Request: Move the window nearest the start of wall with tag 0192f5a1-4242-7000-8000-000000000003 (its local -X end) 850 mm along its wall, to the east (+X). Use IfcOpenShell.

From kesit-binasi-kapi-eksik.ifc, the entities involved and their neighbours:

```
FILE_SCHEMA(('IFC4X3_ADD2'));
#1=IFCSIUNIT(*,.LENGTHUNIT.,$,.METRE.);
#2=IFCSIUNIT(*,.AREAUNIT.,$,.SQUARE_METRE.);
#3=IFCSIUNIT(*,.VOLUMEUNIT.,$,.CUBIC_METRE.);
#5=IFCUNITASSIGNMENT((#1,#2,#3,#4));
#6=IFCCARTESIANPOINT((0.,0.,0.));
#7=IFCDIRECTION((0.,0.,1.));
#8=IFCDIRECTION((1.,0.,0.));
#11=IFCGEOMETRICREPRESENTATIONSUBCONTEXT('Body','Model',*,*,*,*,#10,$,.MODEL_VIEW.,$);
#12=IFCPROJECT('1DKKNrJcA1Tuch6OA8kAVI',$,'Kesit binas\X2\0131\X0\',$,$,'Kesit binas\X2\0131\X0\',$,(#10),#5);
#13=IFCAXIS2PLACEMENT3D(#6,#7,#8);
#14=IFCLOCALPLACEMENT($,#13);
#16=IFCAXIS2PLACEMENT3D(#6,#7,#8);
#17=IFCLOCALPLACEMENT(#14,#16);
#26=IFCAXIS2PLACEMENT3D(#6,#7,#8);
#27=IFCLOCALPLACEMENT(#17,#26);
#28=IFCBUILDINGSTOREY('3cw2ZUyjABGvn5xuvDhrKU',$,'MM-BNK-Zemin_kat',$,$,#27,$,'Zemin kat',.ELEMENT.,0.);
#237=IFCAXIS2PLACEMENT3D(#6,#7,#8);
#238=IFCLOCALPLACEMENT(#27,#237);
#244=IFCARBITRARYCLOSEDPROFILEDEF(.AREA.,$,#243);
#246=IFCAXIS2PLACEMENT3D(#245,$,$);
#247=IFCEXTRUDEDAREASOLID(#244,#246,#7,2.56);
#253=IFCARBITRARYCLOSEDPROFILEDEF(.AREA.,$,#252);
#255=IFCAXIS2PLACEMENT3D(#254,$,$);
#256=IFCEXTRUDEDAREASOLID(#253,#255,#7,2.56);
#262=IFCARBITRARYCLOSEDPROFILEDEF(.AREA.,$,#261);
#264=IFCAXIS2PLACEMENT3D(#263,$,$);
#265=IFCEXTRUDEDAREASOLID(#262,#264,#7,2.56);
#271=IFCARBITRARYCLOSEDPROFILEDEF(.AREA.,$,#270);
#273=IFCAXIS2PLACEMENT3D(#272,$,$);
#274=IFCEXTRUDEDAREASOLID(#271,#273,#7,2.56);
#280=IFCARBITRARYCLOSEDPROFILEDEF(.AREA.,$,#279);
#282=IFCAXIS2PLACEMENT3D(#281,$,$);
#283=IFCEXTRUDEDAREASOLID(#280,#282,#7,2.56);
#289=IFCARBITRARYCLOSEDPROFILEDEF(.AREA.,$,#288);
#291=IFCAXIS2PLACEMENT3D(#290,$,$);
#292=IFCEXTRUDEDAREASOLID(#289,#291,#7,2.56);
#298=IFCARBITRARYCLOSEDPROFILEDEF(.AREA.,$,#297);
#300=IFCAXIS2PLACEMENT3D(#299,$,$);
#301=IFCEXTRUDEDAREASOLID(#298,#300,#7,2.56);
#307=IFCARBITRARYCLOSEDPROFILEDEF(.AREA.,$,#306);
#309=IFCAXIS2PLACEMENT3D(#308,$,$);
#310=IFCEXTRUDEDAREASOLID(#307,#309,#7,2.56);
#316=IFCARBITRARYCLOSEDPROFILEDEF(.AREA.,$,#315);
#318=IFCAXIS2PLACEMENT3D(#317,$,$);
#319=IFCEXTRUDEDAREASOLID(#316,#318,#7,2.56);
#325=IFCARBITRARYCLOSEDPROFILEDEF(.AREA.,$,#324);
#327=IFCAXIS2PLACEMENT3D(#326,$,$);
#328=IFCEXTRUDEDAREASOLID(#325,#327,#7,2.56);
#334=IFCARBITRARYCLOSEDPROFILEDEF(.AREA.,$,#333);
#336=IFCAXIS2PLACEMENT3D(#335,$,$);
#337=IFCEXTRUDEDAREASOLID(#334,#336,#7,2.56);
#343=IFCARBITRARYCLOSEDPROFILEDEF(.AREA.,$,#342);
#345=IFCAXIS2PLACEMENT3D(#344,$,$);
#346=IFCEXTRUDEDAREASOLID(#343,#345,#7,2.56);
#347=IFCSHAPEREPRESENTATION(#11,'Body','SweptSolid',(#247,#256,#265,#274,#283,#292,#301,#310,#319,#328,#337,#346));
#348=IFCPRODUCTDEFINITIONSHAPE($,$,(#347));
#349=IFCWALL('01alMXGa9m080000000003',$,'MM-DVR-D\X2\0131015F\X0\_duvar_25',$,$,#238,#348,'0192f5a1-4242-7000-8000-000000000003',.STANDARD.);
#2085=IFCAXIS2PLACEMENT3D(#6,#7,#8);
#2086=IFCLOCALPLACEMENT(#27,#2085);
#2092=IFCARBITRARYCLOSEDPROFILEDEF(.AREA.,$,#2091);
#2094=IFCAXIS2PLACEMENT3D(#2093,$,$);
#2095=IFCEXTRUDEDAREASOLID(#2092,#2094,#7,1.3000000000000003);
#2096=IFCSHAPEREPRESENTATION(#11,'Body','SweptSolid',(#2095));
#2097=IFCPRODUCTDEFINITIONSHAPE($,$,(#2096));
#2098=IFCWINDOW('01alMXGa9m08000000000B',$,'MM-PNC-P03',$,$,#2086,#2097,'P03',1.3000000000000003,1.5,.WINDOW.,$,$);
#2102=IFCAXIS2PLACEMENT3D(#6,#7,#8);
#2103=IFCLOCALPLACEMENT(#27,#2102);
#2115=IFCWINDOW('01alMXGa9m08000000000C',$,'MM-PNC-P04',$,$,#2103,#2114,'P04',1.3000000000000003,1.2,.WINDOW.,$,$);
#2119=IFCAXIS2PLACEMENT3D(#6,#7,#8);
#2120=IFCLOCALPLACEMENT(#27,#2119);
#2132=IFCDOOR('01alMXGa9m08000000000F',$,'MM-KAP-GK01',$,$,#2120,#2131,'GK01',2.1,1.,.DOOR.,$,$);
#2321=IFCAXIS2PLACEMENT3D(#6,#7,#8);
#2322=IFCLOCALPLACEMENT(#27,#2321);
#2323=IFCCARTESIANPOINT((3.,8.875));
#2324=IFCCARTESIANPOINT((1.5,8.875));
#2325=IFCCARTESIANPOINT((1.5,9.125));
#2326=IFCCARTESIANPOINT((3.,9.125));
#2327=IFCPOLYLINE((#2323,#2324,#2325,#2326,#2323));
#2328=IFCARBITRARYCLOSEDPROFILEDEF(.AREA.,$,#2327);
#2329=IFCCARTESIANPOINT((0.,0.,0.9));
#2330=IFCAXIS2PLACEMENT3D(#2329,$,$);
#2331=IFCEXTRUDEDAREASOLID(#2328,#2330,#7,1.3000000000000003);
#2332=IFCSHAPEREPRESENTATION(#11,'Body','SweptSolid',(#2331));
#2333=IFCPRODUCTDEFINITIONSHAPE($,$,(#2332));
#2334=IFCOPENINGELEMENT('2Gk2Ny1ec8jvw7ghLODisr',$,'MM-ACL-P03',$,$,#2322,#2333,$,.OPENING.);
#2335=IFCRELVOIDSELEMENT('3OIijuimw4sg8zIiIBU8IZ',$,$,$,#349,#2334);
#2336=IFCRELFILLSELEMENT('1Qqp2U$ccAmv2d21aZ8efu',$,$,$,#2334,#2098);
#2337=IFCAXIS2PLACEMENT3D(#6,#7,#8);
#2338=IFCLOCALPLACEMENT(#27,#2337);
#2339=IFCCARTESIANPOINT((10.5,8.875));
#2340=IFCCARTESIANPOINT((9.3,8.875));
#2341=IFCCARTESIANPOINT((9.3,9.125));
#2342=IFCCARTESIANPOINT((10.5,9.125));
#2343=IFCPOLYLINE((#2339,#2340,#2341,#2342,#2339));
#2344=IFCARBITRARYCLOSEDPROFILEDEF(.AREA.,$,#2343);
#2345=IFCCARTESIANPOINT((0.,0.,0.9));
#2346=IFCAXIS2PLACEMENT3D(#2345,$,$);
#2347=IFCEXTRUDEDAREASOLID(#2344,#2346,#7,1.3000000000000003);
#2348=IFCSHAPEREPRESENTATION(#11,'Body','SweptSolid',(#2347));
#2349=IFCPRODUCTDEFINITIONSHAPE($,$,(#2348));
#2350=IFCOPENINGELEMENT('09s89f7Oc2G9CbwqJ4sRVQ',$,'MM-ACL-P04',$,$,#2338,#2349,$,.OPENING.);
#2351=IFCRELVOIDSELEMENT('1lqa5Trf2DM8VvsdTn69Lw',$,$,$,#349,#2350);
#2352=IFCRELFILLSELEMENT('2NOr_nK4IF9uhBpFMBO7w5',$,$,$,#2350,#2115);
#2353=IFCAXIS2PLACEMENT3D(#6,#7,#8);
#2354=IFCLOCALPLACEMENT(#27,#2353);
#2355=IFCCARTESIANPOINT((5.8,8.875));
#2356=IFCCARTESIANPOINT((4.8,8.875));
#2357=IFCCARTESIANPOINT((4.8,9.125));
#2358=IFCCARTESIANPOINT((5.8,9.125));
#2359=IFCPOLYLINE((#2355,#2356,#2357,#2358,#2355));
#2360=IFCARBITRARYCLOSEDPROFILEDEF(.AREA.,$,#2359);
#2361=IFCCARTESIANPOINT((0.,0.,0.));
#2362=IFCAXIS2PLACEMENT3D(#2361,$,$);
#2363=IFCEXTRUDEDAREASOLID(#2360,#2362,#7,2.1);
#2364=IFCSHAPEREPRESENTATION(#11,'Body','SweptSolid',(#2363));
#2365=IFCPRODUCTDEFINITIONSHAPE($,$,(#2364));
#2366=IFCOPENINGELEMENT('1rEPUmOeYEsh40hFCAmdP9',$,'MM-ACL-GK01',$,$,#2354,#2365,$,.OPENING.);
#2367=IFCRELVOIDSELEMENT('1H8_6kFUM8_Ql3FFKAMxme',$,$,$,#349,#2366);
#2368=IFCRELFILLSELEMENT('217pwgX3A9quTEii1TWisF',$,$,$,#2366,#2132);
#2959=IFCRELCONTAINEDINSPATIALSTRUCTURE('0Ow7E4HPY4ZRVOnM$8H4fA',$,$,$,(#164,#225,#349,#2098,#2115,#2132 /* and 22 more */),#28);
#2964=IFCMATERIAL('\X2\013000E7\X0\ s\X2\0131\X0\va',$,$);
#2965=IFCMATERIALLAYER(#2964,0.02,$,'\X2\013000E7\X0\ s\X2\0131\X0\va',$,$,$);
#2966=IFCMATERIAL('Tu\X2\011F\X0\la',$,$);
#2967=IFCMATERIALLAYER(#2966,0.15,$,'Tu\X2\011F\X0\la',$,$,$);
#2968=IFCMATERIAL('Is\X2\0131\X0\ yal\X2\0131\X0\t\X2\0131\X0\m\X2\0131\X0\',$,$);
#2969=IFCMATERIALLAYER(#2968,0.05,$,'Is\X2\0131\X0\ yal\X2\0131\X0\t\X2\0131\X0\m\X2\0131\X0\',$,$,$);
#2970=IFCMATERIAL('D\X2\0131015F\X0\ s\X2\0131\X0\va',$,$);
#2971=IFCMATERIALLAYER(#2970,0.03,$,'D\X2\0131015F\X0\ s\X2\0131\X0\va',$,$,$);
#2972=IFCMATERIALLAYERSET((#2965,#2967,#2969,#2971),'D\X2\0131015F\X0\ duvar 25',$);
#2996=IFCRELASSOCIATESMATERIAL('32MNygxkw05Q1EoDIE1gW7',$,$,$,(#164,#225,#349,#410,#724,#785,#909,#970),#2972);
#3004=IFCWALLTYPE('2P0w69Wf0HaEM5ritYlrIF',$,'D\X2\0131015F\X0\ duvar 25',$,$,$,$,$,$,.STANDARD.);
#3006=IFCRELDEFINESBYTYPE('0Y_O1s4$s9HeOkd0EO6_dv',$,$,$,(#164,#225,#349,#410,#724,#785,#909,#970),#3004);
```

```python
import ifcopenshell
import ifcopenshell.api.geometry
import ifcopenshell.util.placement
import ifcopenshell.util.unit

model = ifcopenshell.open("kesit-binasi-kapi-eksik.ifc")
unit_scale = ifcopenshell.util.unit.calculate_unit_scale(model)

window = model.by_id(2098)
opening = window.FillsVoids[0].RelatingOpeningElement
wall = opening.VoidsElements[0].RelatingBuildingElement

wall_matrix = ifcopenshell.util.placement.get_local_placement(wall.ObjectPlacement)
shift = wall_matrix[:3, 0] * 0.85 / unit_scale
before = ifcopenshell.util.placement.get_local_placement(window.ObjectPlacement)[:3, 3].copy()

# The window is not placed relative to its opening, so move both.
for product in (opening, window):
    matrix = ifcopenshell.util.placement.get_local_placement(product.ObjectPlacement)
    matrix[:3, 3] += shift
    ifcopenshell.api.geometry.edit_object_placement(model, product=product, matrix=matrix, is_si=False)

after = ifcopenshell.util.placement.get_local_placement(window.ObjectPlacement)[:3, 3]
print("window moved by", (after - before).round(3) + 0.0)

model.write("kesit-binasi-kapi-eksik_updated.ifc")
```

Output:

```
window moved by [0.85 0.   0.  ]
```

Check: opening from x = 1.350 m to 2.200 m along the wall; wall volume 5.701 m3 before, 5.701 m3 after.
